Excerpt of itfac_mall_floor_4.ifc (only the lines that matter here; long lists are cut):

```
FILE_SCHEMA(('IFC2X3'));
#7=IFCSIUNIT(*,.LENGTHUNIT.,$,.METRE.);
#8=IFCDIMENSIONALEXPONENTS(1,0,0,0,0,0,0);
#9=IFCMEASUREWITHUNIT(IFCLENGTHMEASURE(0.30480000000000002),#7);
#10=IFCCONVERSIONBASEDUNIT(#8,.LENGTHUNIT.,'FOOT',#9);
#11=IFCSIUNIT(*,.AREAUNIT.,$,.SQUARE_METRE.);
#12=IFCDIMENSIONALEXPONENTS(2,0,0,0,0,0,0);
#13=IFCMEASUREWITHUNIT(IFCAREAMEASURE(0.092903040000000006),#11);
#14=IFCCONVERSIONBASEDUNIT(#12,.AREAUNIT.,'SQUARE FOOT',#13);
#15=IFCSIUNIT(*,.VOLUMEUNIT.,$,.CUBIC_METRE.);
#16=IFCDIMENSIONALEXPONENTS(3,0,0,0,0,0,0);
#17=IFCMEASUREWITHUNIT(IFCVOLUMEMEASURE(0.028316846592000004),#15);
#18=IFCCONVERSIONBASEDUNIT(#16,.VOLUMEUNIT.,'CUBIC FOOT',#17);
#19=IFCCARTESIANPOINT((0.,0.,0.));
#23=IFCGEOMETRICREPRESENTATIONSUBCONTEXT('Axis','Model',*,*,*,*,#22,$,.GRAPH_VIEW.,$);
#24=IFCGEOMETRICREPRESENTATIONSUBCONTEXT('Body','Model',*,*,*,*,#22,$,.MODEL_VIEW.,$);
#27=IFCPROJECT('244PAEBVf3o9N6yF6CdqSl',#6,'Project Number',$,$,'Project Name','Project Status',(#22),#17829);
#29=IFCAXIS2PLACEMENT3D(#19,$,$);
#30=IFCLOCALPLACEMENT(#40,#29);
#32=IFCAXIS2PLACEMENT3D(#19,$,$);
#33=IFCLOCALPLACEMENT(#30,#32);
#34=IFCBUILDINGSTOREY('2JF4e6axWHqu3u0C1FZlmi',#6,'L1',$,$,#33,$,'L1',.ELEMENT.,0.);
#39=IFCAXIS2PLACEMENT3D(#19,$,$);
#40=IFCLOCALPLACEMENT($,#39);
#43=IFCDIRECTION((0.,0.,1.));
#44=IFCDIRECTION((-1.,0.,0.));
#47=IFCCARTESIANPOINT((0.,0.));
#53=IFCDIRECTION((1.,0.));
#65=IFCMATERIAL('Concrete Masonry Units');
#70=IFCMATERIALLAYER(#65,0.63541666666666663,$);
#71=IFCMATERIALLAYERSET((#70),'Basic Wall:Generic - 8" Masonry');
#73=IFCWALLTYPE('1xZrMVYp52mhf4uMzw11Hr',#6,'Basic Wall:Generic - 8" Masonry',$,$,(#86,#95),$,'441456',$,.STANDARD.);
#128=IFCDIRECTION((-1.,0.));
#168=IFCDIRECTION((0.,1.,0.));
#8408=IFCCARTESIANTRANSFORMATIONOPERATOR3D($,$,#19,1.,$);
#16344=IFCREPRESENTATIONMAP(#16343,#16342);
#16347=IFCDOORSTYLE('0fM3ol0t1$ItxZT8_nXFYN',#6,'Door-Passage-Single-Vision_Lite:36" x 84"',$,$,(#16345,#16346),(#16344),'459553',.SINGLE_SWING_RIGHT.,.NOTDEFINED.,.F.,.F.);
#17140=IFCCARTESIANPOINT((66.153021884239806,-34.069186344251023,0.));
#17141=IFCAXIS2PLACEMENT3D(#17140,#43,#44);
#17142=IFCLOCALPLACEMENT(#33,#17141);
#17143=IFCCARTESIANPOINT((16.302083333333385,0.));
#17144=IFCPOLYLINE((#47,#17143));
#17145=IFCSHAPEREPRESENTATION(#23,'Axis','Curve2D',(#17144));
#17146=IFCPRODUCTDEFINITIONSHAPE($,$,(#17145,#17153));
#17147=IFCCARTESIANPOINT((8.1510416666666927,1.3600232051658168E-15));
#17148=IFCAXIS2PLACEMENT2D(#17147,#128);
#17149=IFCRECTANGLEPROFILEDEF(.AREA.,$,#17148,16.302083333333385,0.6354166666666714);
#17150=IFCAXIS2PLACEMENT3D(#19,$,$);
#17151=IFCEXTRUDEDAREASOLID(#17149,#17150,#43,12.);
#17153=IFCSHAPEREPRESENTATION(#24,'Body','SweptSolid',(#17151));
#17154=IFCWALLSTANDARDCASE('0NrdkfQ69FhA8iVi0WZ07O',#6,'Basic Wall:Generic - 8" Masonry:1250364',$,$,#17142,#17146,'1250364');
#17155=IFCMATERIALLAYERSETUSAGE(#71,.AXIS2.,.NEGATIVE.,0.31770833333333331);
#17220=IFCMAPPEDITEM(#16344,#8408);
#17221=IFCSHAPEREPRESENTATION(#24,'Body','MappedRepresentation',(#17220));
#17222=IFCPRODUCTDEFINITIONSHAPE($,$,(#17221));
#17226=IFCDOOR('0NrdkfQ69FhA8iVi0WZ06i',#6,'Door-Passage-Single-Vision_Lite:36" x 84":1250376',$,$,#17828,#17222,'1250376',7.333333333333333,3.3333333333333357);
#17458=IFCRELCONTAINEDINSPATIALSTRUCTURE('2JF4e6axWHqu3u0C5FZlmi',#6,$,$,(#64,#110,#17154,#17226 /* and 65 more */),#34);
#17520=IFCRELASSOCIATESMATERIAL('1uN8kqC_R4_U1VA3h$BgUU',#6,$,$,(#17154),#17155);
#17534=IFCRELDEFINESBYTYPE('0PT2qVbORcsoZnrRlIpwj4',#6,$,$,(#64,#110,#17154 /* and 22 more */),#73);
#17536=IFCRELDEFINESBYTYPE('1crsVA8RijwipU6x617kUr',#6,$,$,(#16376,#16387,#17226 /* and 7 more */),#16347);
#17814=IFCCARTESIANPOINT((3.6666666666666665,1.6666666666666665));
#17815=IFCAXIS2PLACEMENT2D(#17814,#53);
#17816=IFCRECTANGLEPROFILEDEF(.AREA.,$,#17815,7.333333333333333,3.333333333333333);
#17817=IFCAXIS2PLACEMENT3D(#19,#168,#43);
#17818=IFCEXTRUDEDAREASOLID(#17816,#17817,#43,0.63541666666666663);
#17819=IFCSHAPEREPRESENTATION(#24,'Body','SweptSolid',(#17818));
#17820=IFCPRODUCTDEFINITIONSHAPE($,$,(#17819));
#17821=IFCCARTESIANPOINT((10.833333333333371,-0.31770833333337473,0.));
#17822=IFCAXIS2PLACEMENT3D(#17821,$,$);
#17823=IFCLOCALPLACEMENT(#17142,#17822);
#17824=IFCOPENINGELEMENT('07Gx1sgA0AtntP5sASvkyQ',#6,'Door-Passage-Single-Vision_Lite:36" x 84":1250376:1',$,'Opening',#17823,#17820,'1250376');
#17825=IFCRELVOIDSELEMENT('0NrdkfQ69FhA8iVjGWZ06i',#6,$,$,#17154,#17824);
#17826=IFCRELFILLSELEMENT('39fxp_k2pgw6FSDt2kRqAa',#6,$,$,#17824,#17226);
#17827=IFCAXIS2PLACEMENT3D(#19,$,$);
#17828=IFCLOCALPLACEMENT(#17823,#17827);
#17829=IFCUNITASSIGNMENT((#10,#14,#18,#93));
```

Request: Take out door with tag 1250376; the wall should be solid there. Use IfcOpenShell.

```python
import ifcopenshell
import ifcopenshell.api.feature
import ifcopenshell.api.root
import ifcopenshell.geom
import ifcopenshell.util.shape

model = ifcopenshell.open("itfac_mall_floor_4.ifc")
settings = ifcopenshell.geom.settings()


def volume(element):
    """Net volume in cubic metres, openings subtracted."""
    shape = ifcopenshell.geom.create_shape(settings, element)
    return ifcopenshell.util.shape.get_volume(shape.geometry)


door = model.by_guid("0NrdkfQ69FhA8iVi0WZ06i")
opening = door.FillsVoids[0].RelatingOpeningElement
wall = opening.VoidsElements[0].RelatingBuildingElement
before = volume(wall)

ifcopenshell.api.root.remove_product(model, product=door)
ifcopenshell.api.feature.remove_feature(model, feature=opening)

after = volume(wall)

print(f"wall volume {before:.3f} -> {after:.3f} m3")

model.write("itfac_mall_floor_4_updated.ifc")
```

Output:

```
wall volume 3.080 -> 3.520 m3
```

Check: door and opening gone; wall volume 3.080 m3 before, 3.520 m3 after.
